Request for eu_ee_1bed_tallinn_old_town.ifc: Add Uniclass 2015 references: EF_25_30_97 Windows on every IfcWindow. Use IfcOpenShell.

First a look at what the model holds.

```python
import ifcopenshell

model = ifcopenshell.open("eu_ee_1bed_tallinn_old_town.ifc")
print(model.schema)
print("classifications:", [c.Name for c in model.by_type("IfcClassification")])
for ifc_class in ("IfcDoor", "IfcRoof", "IfcStair", "IfcWall", "IfcWindow"):
    print(ifc_class, len(model.by_type(ifc_class)))
```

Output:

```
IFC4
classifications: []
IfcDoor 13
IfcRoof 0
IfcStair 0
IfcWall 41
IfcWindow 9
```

```python
import ifcopenshell
import ifcopenshell.api.classification

model = ifcopenshell.open("eu_ee_1bed_tallinn_old_town.ifc")

system = ifcopenshell.api.classification.add_classification(model, classification="Uniclass 2015")

codes = {
    "IfcWindow": ("EF_25_30_97", "Windows"),
}
for ifc_class, (code, name) in codes.items():
    products = model.by_type(ifc_class)
    ifcopenshell.api.classification.add_reference(
        model, products=products, classification=system, identification=code, name=name
    )
    print(code, len(products))

model.write("eu_ee_1bed_tallinn_old_town_rev.ifc")
```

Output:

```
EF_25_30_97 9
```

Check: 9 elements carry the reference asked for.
